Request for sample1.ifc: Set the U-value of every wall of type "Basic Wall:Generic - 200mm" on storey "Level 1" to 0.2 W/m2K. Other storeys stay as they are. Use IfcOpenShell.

First a look at what the model holds.

```python
import ifcopenshell
import ifcopenshell.util.element

model = ifcopenshell.open("sample1.ifc")
print(model.schema)
storey = next(s for s in model.by_type("IfcBuildingStorey") if s.Name == "Level 1")
walls = [e for e in ifcopenshell.util.element.get_decomposition(storey) if e.is_a("IfcWall")]
seen = {}
for e in walls:
    element_type = ifcopenshell.util.element.get_type(e)
    key = (element_type.Name if element_type != e and element_type else None, ifcopenshell.util.element.get_pset(e, "Pset_WallCommon", "ThermalTransmittance"))
    seen[key] = seen.get(key, 0) + 1
for (name, value), count in sorted(seen.items(), key=str):
    print(count, "x", name, "|", value)
```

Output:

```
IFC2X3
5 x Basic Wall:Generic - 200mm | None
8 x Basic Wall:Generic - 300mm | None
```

```python
import ifcopenshell
import ifcopenshell.api.pset
import ifcopenshell.util.element

model = ifcopenshell.open("sample1.ifc")

storey = next(s for s in model.by_type("IfcBuildingStorey") if s.Name == "Level 1")
walls = [e for e in ifcopenshell.util.element.get_decomposition(storey) if e.is_a("IfcWall")]

count = 0
for e in walls:
    element_type = ifcopenshell.util.element.get_type(e)
    if element_type in (None, e) or element_type.Name != "Basic Wall:Generic - 200mm":
        continue
    # add_pset returns the element's existing set when there is one.
    pset = ifcopenshell.api.pset.add_pset(model, product=e, name="Pset_WallCommon")
    ifcopenshell.api.pset.edit_pset(model, pset=pset, properties={"ThermalTransmittance": 0.2})
    count += 1

print(count, "walls updated")

model.write("sample1_edited.ifc")
```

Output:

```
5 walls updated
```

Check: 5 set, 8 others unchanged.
